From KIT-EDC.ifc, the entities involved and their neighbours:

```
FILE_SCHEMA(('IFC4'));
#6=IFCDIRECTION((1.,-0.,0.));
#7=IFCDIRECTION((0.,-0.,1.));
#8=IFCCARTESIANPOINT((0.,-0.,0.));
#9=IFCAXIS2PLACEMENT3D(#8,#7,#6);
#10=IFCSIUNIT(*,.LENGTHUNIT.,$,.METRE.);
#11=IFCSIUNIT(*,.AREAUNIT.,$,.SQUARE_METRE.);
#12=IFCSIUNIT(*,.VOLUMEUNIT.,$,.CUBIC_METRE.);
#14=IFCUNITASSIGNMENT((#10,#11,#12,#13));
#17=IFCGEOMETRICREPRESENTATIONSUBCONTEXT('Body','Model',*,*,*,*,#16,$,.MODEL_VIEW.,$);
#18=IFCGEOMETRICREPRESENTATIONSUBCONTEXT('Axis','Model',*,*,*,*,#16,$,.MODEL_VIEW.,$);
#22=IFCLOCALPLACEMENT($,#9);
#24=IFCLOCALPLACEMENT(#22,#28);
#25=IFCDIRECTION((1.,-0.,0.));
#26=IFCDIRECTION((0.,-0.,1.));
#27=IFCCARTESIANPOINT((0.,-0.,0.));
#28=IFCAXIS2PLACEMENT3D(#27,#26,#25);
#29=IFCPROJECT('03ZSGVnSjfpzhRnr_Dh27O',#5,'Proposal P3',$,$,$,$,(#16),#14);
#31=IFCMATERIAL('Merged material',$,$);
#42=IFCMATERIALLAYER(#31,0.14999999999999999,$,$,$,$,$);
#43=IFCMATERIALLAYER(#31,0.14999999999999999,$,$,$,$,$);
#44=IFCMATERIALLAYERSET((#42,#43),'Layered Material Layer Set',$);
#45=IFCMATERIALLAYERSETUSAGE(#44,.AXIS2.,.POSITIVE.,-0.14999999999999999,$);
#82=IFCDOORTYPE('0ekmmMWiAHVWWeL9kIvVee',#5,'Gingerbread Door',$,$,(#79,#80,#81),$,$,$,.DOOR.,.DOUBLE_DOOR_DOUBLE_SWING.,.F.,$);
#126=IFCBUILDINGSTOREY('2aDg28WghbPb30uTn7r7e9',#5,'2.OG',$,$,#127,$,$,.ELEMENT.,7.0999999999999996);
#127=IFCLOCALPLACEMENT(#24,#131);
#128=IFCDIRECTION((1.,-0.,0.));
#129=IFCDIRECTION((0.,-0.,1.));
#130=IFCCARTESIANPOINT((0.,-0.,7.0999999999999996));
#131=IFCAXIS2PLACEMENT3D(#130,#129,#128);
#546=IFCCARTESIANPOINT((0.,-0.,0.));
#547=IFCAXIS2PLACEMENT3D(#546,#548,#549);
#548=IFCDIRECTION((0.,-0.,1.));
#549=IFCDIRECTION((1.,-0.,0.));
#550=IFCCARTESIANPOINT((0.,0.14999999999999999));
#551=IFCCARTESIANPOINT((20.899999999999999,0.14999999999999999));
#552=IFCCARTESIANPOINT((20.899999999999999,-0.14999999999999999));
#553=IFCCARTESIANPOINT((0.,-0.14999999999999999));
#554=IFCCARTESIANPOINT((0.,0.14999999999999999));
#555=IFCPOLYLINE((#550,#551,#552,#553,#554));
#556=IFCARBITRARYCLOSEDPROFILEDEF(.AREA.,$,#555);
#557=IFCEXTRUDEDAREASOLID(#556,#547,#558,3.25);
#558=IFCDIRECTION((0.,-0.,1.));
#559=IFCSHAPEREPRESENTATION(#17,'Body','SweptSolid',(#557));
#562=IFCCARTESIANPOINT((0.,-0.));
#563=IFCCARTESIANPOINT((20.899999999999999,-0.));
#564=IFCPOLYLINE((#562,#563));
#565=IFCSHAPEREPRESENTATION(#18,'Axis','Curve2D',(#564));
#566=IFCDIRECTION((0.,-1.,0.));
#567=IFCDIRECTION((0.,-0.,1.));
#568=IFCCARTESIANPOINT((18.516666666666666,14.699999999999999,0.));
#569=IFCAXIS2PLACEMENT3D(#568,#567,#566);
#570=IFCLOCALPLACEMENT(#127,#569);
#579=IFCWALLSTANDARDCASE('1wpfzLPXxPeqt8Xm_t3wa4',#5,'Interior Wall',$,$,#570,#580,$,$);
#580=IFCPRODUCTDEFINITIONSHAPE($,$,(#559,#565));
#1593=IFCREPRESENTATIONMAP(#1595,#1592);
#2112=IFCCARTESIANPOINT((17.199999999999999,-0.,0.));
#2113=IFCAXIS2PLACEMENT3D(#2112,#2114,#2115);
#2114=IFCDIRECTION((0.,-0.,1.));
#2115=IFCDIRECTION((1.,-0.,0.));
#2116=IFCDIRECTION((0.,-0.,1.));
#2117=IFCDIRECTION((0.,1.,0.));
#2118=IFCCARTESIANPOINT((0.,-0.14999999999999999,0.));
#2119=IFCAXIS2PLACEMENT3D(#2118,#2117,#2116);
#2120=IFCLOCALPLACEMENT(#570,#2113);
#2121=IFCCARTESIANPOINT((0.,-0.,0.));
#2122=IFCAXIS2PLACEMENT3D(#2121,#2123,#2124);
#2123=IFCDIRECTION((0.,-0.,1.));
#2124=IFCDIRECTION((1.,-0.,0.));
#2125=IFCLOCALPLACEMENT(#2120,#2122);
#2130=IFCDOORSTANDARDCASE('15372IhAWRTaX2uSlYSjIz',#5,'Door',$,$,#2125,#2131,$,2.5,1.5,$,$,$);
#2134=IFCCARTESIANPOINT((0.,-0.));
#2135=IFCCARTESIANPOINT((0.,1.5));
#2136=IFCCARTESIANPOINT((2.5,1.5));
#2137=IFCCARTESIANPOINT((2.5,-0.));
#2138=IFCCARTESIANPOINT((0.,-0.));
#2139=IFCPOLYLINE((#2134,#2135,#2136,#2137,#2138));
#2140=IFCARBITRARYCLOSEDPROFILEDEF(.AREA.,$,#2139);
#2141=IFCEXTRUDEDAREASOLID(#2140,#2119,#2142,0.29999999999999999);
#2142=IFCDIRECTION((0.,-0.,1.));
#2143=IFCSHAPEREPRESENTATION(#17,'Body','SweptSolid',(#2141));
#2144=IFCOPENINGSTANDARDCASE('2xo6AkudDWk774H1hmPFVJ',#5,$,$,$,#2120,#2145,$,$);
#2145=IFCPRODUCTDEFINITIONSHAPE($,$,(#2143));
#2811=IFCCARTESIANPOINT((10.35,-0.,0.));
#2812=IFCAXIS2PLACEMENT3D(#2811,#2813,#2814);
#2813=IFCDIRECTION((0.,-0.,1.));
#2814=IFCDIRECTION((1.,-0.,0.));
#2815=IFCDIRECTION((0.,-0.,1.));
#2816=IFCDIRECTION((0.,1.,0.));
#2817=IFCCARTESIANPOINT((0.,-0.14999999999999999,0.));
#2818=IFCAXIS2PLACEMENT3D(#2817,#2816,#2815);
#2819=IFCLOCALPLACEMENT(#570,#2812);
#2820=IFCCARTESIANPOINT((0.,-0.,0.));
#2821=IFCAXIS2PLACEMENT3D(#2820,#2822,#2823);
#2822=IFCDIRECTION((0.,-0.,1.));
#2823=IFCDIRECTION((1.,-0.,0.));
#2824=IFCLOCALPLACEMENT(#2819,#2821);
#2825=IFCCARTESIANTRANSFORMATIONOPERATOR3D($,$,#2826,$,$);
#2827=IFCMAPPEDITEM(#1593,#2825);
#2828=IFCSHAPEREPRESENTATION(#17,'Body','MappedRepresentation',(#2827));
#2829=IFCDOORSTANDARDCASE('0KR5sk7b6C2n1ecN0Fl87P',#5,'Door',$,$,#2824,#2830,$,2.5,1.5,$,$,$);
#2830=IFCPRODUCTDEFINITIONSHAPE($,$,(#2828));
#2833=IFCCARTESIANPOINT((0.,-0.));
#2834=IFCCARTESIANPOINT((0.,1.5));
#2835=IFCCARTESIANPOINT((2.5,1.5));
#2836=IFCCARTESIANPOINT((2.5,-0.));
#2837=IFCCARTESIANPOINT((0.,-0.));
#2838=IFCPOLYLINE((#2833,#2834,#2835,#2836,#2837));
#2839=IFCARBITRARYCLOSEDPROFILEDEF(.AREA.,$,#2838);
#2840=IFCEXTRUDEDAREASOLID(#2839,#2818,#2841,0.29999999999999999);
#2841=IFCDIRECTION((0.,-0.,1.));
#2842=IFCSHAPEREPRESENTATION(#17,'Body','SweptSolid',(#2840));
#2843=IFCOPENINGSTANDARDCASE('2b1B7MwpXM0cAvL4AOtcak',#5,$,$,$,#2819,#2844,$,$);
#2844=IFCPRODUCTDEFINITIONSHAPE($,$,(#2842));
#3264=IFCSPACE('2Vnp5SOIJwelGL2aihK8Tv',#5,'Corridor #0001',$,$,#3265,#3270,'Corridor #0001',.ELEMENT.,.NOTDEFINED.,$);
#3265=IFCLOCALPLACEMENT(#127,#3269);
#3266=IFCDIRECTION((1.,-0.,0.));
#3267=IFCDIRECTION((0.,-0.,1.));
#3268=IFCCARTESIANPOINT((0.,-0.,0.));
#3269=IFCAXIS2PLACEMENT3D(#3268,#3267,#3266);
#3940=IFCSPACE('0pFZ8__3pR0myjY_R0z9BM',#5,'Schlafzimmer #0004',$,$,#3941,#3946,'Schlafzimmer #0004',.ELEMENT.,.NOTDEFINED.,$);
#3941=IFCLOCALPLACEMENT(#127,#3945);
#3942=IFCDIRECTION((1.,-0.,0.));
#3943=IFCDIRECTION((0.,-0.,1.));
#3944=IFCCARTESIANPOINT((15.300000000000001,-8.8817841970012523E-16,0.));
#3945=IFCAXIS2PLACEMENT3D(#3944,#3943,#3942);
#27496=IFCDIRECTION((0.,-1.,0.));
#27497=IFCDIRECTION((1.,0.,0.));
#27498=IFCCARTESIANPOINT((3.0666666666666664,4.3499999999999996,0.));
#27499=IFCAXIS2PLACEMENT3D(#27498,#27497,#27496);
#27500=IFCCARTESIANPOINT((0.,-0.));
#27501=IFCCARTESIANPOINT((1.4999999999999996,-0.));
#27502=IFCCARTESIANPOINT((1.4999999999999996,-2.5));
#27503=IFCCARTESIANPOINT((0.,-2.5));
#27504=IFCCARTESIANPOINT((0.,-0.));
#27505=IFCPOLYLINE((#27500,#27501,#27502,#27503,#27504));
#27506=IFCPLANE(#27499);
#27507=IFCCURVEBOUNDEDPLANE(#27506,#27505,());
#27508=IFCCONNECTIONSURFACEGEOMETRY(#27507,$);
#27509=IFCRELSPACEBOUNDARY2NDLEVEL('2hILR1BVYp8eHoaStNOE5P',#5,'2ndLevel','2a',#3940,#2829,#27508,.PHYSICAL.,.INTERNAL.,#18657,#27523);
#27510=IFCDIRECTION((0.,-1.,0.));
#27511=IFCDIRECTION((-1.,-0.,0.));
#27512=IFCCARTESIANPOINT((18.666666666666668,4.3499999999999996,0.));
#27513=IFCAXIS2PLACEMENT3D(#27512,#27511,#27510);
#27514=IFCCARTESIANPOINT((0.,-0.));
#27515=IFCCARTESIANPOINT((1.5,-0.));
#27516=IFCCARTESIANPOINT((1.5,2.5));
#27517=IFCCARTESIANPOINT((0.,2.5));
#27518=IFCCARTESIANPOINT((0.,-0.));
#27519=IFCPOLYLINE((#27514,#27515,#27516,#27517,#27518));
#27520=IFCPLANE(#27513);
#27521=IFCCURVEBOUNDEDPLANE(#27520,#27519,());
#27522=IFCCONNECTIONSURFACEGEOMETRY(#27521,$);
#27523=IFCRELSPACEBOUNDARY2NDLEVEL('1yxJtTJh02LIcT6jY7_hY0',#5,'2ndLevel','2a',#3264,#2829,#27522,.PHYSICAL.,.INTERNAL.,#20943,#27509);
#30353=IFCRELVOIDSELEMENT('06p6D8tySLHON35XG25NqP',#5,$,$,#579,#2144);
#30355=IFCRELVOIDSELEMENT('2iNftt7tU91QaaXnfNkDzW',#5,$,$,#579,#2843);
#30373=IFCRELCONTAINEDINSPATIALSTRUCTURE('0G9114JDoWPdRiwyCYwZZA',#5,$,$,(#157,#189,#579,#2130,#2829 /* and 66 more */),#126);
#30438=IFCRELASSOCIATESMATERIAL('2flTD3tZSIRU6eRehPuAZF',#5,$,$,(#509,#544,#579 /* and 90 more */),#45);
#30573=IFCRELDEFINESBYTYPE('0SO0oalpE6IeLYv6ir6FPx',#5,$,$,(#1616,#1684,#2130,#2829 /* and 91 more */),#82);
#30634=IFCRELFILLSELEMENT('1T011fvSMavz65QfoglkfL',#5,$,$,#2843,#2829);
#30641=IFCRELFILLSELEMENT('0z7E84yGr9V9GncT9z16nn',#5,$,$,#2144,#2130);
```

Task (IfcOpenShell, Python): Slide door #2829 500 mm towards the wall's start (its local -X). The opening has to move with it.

```python
import numpy as np
import ifcopenshell
import ifcopenshell.api.geometry
import ifcopenshell.util.placement

model = ifcopenshell.open("KIT-EDC.ifc")

door = model.by_guid("0KR5sk7b6C2n1ecN0Fl87P")
opening = door.FillsVoids[0].RelatingOpeningElement
wall = opening.VoidsElements[0].RelatingBuildingElement

wall_matrix = ifcopenshell.util.placement.get_local_placement(wall.ObjectPlacement)
shift = wall_matrix[:3, 0] * -0.5
before = ifcopenshell.util.placement.get_local_placement(door.ObjectPlacement)[:3, 3].copy()

# The door is placed relative to its opening, so it follows when the opening moves.
matrix = ifcopenshell.util.placement.get_local_placement(opening.ObjectPlacement)
matrix[:3, 3] += shift
ifcopenshell.api.geometry.edit_object_placement(
    model, product=opening, matrix=matrix, is_si=False, should_transform_children=True
)

# Space boundary surfaces are stored in each space's coordinates; move them too.
for rel in door.ProvidesBoundaries:
    if not rel.ConnectionGeometry:
        continue
    surface = rel.ConnectionGeometry.SurfaceOnRelatingElement.BasisSurface
    space_matrix = ifcopenshell.util.placement.get_local_placement(rel.RelatingSpace.ObjectPlacement)
    point = np.array(surface.Position.Location.Coordinates) + space_matrix[:3, :3].T @ shift
    surface.Position = model.createIfcAxis2Placement3D(
        model.createIfcCartesianPoint(point.tolist()), surface.Position.Axis, surface.Position.RefDirection
    )

after = ifcopenshell.util.placement.get_local_placement(door.ObjectPlacement)[:3, 3]
print("door moved by", (after - before).round(3) + 0.0)

model.write("KIT-EDC_rev.ifc")
```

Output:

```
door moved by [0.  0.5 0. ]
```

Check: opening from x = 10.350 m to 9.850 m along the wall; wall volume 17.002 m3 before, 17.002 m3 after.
